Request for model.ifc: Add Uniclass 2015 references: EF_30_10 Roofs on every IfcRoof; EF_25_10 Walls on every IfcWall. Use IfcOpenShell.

First a look at what the model holds.

```python
import ifcopenshell

model = ifcopenshell.open("model.ifc")
print(model.schema)
print("classifications:", [c.Name for c in model.by_type("IfcClassification")])
for ifc_class in ("IfcDoor", "IfcRoof", "IfcStair", "IfcWall", "IfcWindow"):
    print(ifc_class, len(model.by_type(ifc_class)))
```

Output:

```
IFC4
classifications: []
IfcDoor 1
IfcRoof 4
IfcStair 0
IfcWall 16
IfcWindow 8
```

```python
import ifcopenshell
import ifcopenshell.api.classification

model = ifcopenshell.open("model.ifc")

system = ifcopenshell.api.classification.add_classification(model, classification="Uniclass 2015")

codes = {
    "IfcRoof": ("EF_30_10", "Roofs"),
    "IfcWall": ("EF_25_10", "Walls"),
}
for ifc_class, (code, name) in codes.items():
    products = model.by_type(ifc_class)
    ifcopenshell.api.classification.add_reference(
        model, products=products, classification=system, identification=code, name=name
    )
    print(code, len(products))

model.write("model_edited.ifc")
```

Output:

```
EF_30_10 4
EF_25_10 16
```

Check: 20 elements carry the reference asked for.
